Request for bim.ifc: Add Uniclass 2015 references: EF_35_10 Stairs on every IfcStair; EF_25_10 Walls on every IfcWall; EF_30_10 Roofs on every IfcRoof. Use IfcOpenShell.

First a look at what the model holds.

```python
import ifcopenshell

model = ifcopenshell.open("bim.ifc")
print(model.schema)
print("classifications:", [c.Name for c in model.by_type("IfcClassification")])
for ifc_class in ("IfcDoor", "IfcRoof", "IfcStair", "IfcWall", "IfcWindow"):
    print(ifc_class, len(model.by_type(ifc_class)))
```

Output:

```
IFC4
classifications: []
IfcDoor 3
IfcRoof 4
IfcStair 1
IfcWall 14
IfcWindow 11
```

```python
import ifcopenshell
import ifcopenshell.api.classification

model = ifcopenshell.open("bim.ifc")

system = ifcopenshell.api.classification.add_classification(model, classification="Uniclass 2015")

codes = {
    "IfcStair": ("EF_35_10", "Stairs"),
    "IfcWall": ("EF_25_10", "Walls"),
    "IfcRoof": ("EF_30_10", "Roofs"),
}
for ifc_class, (code, name) in codes.items():
    products = model.by_type(ifc_class)
    ifcopenshell.api.classification.add_reference(
        model, products=products, classification=system, identification=code, name=name
    )
    print(code, len(products))

model.write("bim_rev.ifc")
```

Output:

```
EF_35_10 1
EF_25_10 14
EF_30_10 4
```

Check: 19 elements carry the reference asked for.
